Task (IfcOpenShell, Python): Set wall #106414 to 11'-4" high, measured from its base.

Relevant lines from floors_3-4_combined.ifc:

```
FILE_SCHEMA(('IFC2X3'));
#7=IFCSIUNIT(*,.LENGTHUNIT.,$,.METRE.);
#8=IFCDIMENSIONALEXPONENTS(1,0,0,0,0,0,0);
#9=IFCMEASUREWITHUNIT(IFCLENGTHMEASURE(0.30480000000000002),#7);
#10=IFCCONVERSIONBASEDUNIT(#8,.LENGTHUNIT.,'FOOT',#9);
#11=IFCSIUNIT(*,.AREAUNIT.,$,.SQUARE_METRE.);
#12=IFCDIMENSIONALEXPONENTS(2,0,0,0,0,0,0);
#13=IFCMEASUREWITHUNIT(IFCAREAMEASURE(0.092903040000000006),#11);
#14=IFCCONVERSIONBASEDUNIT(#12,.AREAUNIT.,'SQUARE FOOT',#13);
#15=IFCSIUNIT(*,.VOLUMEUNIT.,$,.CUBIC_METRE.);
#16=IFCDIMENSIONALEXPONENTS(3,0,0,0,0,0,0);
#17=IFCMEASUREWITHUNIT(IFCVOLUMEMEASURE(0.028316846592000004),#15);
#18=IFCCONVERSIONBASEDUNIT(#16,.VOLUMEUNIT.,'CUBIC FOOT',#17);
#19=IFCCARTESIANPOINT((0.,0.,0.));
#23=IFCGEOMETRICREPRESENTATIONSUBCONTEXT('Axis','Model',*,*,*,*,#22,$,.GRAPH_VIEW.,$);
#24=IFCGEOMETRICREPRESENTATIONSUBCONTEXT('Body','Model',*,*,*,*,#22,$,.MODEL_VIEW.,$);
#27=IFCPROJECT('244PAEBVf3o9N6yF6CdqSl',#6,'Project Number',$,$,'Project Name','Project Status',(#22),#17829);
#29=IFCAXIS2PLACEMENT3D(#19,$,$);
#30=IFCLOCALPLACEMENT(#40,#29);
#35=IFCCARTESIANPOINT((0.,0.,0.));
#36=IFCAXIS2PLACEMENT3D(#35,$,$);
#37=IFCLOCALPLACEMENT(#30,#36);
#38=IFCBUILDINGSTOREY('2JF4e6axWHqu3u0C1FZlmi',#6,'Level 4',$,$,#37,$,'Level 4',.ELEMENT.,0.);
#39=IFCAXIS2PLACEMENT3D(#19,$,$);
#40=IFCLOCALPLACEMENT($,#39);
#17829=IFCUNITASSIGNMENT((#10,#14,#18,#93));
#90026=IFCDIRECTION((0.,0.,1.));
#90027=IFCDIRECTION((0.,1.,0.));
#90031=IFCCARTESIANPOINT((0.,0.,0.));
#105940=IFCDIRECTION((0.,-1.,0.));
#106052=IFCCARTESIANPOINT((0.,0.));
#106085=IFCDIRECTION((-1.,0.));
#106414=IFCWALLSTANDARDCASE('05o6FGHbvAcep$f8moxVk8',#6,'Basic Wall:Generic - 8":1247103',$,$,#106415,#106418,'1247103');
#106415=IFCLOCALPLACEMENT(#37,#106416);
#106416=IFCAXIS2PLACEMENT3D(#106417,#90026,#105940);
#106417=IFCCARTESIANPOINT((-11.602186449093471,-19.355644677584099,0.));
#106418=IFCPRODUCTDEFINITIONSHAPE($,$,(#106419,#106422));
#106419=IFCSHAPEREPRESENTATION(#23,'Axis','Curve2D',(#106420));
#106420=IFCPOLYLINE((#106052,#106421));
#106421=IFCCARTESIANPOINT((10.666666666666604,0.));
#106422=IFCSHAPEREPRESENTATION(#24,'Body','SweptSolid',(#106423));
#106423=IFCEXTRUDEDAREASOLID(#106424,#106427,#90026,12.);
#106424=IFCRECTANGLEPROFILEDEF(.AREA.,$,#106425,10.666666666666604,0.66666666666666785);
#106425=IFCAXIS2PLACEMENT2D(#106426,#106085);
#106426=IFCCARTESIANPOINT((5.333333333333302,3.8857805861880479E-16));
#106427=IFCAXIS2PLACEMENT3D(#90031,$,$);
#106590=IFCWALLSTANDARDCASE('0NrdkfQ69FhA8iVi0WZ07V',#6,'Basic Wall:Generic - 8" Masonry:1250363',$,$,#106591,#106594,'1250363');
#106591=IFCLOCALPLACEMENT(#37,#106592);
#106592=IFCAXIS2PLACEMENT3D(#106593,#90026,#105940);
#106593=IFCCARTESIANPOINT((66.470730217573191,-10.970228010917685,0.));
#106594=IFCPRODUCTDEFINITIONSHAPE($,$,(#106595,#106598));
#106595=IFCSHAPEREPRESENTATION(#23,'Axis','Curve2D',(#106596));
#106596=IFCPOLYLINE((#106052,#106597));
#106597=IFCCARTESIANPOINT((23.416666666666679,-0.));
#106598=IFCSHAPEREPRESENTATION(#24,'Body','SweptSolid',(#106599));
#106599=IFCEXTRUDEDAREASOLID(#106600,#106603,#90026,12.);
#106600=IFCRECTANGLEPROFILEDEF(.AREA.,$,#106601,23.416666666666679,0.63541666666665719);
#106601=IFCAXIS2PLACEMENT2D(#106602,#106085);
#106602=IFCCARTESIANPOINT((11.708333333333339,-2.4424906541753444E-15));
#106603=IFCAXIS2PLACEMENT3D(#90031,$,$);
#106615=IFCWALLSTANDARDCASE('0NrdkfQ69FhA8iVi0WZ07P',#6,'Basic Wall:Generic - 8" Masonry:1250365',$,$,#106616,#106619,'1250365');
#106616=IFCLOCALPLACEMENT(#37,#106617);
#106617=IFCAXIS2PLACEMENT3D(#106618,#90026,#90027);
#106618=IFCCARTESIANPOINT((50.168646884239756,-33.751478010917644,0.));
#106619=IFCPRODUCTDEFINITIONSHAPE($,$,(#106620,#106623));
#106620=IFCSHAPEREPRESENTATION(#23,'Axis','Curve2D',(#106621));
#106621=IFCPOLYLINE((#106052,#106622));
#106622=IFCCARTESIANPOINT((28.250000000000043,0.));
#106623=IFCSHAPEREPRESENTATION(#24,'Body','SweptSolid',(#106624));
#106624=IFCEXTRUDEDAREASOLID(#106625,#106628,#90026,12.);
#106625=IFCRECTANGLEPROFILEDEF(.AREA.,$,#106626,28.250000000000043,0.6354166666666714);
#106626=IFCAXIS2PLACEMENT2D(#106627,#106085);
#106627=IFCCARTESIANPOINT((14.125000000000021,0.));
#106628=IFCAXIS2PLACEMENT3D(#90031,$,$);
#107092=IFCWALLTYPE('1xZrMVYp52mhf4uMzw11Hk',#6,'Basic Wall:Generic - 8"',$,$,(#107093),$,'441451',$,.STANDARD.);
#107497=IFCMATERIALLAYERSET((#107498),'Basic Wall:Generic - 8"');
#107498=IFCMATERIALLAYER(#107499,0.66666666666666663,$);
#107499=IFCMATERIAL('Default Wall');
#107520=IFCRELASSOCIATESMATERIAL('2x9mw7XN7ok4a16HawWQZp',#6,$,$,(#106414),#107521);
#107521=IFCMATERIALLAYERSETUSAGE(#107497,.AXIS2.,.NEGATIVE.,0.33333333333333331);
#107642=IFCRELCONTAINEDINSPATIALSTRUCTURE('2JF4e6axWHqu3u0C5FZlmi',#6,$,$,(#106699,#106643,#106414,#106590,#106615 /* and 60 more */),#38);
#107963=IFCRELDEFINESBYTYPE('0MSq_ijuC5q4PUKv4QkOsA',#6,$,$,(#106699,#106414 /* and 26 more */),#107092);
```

```python
import ifcopenshell
import ifcopenshell.geom
import ifcopenshell.util.representation
import ifcopenshell.util.shape
import ifcopenshell.util.unit

model = ifcopenshell.open("floors_3-4_combined.ifc")
unit_scale = ifcopenshell.util.unit.calculate_unit_scale(model)
settings = ifcopenshell.geom.settings()


def volume(element):
    """Net volume in cubic metres, openings subtracted."""
    shape = ifcopenshell.geom.create_shape(settings, element)
    return ifcopenshell.util.shape.get_volume(shape.geometry)


wall = model.by_guid("05o6FGHbvAcep$f8moxVk8")
before = volume(wall)

body = ifcopenshell.util.representation.get_representation(wall, "Model", "Body")
solid = body.Items[0]
old_height = solid.Depth
solid.Depth = 136 * 0.0254 / unit_scale
after = volume(wall)

print(f"height {old_height:g} -> {solid.Depth:g}, volume {before:.3f} -> {after:.3f} m3")

model.write("floors_3-4_combined_edited.ifc")
```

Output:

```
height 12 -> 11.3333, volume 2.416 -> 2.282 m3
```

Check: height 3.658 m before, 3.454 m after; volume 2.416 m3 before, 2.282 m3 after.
